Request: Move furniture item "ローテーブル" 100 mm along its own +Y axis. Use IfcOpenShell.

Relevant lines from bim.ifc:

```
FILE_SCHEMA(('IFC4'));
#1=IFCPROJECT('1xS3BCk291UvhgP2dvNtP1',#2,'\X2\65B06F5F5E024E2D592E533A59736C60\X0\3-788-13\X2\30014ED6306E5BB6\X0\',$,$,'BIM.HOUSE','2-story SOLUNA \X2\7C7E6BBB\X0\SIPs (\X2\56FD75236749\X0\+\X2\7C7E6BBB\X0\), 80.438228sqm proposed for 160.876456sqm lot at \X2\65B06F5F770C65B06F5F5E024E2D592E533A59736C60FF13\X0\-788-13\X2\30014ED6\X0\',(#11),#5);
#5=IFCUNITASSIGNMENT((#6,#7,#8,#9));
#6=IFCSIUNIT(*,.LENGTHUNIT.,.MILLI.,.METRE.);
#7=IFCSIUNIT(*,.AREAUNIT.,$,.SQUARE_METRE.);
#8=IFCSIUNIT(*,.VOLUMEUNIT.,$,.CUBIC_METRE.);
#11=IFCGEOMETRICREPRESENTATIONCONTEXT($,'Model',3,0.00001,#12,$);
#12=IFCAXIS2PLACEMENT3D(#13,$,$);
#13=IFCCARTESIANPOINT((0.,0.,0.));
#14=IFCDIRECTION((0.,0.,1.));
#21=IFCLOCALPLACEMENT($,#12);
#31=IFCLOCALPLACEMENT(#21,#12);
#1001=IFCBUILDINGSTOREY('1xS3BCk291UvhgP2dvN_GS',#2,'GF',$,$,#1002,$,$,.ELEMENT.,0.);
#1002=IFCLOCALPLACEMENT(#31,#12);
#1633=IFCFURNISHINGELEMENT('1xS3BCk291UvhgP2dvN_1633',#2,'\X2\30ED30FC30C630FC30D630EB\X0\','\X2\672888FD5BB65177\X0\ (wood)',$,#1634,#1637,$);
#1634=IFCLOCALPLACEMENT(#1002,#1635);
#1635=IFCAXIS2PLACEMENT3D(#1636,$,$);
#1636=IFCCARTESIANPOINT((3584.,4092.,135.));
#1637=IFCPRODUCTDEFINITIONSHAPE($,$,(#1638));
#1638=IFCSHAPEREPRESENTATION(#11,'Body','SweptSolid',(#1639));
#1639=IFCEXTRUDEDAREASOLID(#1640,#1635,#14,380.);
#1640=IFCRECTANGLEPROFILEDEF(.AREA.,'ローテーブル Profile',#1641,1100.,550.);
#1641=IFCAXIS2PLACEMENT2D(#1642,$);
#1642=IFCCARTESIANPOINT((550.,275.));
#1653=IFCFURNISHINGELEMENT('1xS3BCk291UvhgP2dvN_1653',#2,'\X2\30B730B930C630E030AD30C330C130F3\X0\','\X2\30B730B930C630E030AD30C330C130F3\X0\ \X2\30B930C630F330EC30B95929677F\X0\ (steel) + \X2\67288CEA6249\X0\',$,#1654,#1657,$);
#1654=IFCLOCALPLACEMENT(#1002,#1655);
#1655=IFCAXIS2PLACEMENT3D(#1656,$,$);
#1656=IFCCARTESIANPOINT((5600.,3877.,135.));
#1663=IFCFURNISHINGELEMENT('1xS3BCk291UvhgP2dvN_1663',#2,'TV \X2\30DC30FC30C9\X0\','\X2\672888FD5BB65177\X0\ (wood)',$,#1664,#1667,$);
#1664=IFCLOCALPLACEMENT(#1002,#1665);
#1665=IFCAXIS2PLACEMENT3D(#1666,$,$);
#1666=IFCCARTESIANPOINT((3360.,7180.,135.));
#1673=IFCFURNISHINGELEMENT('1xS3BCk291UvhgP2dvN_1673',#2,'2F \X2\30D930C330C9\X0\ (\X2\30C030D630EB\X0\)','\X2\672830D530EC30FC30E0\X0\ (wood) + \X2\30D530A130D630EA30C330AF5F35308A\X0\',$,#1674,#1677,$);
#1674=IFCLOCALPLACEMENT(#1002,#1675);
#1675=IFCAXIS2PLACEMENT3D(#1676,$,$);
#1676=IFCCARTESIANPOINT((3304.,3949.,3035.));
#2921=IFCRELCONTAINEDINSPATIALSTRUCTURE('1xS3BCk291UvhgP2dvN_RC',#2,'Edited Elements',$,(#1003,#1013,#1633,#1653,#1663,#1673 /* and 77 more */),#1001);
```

```python
import ifcopenshell
import ifcopenshell.api.geometry
import ifcopenshell.util.placement
import ifcopenshell.util.unit

model = ifcopenshell.open("bim.ifc")
unit_scale = ifcopenshell.util.unit.calculate_unit_scale(model)

item = model.by_guid("1xS3BCk291UvhgP2dvN_1633")
matrix = ifcopenshell.util.placement.get_local_placement(item.ObjectPlacement)
matrix[:3, 3] += matrix[:3, 1] * 0.1 / unit_scale
ifcopenshell.api.geometry.edit_object_placement(model, product=item, matrix=matrix, is_si=False)

print(ifcopenshell.util.placement.get_local_placement(item.ObjectPlacement).round(3) + 0.0)

model.write("bim_edited.ifc")
```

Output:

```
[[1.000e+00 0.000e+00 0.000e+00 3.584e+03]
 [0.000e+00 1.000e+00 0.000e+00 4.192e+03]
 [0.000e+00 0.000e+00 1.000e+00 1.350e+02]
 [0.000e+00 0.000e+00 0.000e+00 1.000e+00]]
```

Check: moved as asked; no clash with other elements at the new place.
